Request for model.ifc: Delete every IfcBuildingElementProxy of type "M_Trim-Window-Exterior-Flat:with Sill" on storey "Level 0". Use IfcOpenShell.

First a look at what the model holds.

```python
import ifcopenshell
import ifcopenshell.util.element

model = ifcopenshell.open("model.ifc")
print(model.schema)
storey = next(s for s in model.by_type("IfcBuildingStorey") if s.Name == "Level 0")
proxies = [e for e in ifcopenshell.util.element.get_decomposition(storey) if e.is_a("IfcBuildingElementProxy")]
seen = {}
for e in proxies:
    element_type = ifcopenshell.util.element.get_type(e)
    name = element_type.Name if element_type not in (None, e) else None
    seen[name] = seen.get(name, 0) + 1
for name, count in sorted(seen.items(), key=str):
    print(count, "x", name)
```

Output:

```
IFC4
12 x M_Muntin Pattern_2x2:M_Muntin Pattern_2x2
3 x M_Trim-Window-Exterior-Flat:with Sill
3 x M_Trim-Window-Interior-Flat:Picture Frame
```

```python
import ifcopenshell
import ifcopenshell.api.root
import ifcopenshell.util.element

model = ifcopenshell.open("model.ifc")

storey = next(s for s in model.by_type("IfcBuildingStorey") if s.Name == "Level 0")
proxies = [e for e in ifcopenshell.util.element.get_decomposition(storey) if e.is_a("IfcBuildingElementProxy")]
targets = [e for e in proxies if (t := ifcopenshell.util.element.get_type(e)) not in (None, e) and t.Name == "M_Trim-Window-Exterior-Flat:with Sill"]

for e in targets:
    ifcopenshell.api.root.remove_product(model, product=e)
print(len(targets), "removed")

model.write("model_edited.ifc")
```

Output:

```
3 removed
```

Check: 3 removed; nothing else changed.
